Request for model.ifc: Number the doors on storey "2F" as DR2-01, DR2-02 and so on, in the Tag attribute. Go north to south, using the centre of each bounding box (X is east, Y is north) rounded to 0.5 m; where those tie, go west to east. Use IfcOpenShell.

First a look at what the model holds.

```python
import ifcopenshell
import ifcopenshell.util.element
import ifcopenshell.util.placement

model = ifcopenshell.open("model.ifc")
print(model.schema)
storey = next(s for s in model.by_type("IfcBuildingStorey") if s.Name == "2F")
doors = [e for e in ifcopenshell.util.element.get_decomposition(storey) if e.is_a("IfcDoor")]
for e in sorted(doors, key=lambda e: e.id()):
    origin = ifcopenshell.util.placement.get_local_placement(e.ObjectPlacement)[:3, 3]
    print(e.id(), e.Tag, e.Name, origin.round(2) + 0.0, sep=" | ")
```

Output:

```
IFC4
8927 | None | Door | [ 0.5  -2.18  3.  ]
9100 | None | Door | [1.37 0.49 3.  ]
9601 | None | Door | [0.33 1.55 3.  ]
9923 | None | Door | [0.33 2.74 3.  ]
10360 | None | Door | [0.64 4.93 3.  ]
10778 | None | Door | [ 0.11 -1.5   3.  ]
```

```python
import ifcopenshell
import ifcopenshell.geom
import ifcopenshell.util.element
import ifcopenshell.util.shape

model = ifcopenshell.open("model.ifc")
settings = ifcopenshell.geom.settings()
settings.set("use-world-coords", True)


def centre(element):
    shape = ifcopenshell.geom.create_shape(settings, element)
    return ifcopenshell.util.shape.get_bbox_centroid(shape.geometry)


storey = next(s for s in model.by_type("IfcBuildingStorey") if s.Name == "2F")
doors = [e for e in ifcopenshell.util.element.get_decomposition(storey) if e.is_a("IfcDoor")]

# Insertion points can sit at a corner or the storey origin, so sort by the geometry (in metres).
centres = {e: centre(e) for e in doors}
doors.sort(key=lambda e: (-round(centres[e][1] / 0.5), centres[e][0]))

for i, e in enumerate(doors, start=1):
    number = f"DR2-{i:02d}"
    e.Tag = number
    print(e.id(), number)

model.write("model_v2.ifc")
```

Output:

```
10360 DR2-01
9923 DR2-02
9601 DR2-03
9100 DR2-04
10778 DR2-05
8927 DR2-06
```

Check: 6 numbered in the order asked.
